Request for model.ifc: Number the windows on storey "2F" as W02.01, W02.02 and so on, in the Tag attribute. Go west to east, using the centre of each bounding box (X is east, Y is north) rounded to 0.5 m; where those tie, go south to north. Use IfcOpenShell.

First a look at what the model holds.

```python
import ifcopenshell
import ifcopenshell.util.element
import ifcopenshell.util.placement

model = ifcopenshell.open("model.ifc")
print(model.schema)
storey = next(s for s in model.by_type("IfcBuildingStorey") if s.Name == "2F")
windows = [e for e in ifcopenshell.util.element.get_decomposition(storey) if e.is_a("IfcWindow")]
for e in sorted(windows, key=lambda e: e.id()):
    origin = ifcopenshell.util.placement.get_local_placement(e.ObjectPlacement)[:3, 3]
    print(e.id(), e.Tag, e.Name, origin.round(2) + 0.0, sep=" | ")
```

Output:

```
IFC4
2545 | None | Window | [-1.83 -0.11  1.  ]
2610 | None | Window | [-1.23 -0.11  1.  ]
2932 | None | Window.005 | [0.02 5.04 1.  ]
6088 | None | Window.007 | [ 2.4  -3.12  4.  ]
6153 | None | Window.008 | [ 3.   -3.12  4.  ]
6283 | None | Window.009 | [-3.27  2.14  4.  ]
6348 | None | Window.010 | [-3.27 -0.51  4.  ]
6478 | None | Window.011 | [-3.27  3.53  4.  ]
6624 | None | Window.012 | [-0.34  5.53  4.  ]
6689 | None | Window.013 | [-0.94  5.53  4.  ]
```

```python
import ifcopenshell
import ifcopenshell.geom
import ifcopenshell.util.element
import ifcopenshell.util.shape

model = ifcopenshell.open("model.ifc")
settings = ifcopenshell.geom.settings()
settings.set("use-world-coords", True)


def centre(element):
    shape = ifcopenshell.geom.create_shape(settings, element)
    return ifcopenshell.util.shape.get_bbox_centroid(shape.geometry)


storey = next(s for s in model.by_type("IfcBuildingStorey") if s.Name == "2F")
windows = [e for e in ifcopenshell.util.element.get_decomposition(storey) if e.is_a("IfcWindow")]

# Insertion points can sit at a corner or the storey origin, so sort by the geometry (in metres).
centres = {e: centre(e) for e in windows}
windows.sort(key=lambda e: (round(centres[e][0] / 0.5), centres[e][1]))

for i, e in enumerate(windows, start=1):
    number = f"W02.{i:02d}"
    e.Tag = number
    print(e.id(), number)

model.write("model_updated.ifc")
```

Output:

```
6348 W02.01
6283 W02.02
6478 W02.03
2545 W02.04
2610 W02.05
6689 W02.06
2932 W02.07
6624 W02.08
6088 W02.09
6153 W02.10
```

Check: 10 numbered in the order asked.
